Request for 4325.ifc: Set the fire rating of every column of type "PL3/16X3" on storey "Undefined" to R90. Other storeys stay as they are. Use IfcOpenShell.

First a look at what the model holds.

```python
import ifcopenshell
import ifcopenshell.util.element

model = ifcopenshell.open("4325.ifc")
print(model.schema)
storey = next(s for s in model.by_type("IfcBuildingStorey") if s.Name == "Undefined")
columns = [e for e in ifcopenshell.util.element.get_decomposition(storey) if e.is_a("IfcColumn")]
seen = {}
for e in columns:
    element_type = ifcopenshell.util.element.get_type(e)
    key = (element_type.Name if element_type != e and element_type else None, ifcopenshell.util.element.get_pset(e, "Pset_ColumnCommon", "FireRating"))
    seen[key] = seen.get(key, 0) + 1
for (name, value), count in sorted(seen.items(), key=str):
    print(count, "x", name, "|", value)
```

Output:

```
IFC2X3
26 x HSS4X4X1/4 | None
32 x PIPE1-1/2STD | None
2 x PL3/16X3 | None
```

```python
import ifcopenshell
import ifcopenshell.api.pset
import ifcopenshell.util.element

model = ifcopenshell.open("4325.ifc")

storey = next(s for s in model.by_type("IfcBuildingStorey") if s.Name == "Undefined")
columns = [e for e in ifcopenshell.util.element.get_decomposition(storey) if e.is_a("IfcColumn")]

count = 0
for e in columns:
    element_type = ifcopenshell.util.element.get_type(e)
    if element_type in (None, e) or element_type.Name != "PL3/16X3":
        continue
    found = ifcopenshell.util.element.get_pset(e, "Pset_ColumnCommon", should_inherit=False)
    if found:
        pset = model.by_id(found["id"])
        if len(ifcopenshell.util.element.get_elements_by_pset(pset)) > 1:
            pset = ifcopenshell.api.pset.unshare_pset(model, products=[e], pset=pset)[0]
    else:
        pset = ifcopenshell.api.pset.add_pset(model, product=e, name="Pset_ColumnCommon")
    ifcopenshell.api.pset.edit_pset(model, pset=pset, properties={"FireRating": "R90"})
    count += 1

print(count, "columns updated")

model.write("4325-out.ifc")
```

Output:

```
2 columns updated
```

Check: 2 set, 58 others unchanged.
